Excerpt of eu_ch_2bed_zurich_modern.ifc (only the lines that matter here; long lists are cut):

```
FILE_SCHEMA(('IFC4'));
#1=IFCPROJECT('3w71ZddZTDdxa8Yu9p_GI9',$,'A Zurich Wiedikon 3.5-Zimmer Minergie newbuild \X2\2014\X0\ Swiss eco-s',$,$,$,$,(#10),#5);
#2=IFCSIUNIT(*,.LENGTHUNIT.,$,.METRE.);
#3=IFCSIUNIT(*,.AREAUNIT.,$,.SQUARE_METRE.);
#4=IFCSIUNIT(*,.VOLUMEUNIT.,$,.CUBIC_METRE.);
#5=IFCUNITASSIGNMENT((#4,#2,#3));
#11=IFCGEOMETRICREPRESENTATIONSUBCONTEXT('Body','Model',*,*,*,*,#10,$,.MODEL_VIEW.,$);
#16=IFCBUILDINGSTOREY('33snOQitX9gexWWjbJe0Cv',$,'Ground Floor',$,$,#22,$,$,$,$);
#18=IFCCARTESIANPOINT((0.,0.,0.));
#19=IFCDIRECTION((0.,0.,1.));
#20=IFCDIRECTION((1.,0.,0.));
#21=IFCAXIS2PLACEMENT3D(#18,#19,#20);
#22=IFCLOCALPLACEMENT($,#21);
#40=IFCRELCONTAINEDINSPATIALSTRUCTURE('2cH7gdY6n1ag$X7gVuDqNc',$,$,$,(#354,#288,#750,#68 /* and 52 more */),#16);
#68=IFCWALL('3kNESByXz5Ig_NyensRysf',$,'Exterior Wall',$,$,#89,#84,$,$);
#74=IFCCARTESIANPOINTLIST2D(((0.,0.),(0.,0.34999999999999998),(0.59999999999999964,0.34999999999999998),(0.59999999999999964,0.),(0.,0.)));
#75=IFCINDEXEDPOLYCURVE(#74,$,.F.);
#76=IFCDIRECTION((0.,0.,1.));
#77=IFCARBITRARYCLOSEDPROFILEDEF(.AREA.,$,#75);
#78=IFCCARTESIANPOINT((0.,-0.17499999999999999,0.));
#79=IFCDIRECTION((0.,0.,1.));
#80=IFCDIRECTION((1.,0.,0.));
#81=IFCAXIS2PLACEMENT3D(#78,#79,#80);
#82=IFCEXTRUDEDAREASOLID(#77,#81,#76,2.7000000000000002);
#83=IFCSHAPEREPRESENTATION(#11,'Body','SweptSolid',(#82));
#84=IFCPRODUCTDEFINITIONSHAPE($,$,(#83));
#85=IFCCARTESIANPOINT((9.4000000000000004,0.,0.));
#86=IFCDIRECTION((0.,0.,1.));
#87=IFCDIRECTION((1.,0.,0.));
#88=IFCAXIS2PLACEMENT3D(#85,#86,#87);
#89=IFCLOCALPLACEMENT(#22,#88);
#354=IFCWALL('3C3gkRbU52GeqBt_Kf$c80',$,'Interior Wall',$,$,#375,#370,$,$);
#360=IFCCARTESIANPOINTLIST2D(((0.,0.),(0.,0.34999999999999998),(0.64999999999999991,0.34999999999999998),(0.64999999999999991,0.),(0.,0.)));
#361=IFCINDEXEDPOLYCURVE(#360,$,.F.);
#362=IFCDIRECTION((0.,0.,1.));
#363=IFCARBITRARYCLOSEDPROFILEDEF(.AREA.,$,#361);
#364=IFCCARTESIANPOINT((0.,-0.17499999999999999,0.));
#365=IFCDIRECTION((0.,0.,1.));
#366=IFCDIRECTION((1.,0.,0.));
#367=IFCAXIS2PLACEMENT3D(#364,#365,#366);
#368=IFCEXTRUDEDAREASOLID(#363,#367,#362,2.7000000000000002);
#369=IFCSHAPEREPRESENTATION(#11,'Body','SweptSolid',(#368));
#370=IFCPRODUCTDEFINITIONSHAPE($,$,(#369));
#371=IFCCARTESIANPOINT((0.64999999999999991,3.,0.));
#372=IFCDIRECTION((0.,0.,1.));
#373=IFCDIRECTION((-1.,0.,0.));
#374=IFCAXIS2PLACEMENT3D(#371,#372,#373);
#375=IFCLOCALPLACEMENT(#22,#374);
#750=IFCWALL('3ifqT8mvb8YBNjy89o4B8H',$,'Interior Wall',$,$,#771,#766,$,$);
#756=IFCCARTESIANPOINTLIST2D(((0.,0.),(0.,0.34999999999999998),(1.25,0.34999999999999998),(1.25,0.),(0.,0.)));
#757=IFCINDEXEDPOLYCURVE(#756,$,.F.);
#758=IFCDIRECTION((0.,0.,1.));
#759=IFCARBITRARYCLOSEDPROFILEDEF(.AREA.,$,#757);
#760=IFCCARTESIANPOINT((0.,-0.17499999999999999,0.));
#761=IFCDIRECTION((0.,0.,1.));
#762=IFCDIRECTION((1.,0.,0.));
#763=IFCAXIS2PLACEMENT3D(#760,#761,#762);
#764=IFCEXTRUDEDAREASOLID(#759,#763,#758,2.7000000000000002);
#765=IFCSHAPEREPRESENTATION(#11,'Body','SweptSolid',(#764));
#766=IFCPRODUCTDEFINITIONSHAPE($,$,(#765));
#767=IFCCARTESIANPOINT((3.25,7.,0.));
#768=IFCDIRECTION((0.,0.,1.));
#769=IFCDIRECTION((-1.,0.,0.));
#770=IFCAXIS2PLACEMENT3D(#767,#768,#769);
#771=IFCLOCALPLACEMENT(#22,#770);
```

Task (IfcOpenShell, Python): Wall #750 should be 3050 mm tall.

```python
import ifcopenshell
import ifcopenshell.geom
import ifcopenshell.util.representation
import ifcopenshell.util.shape
import ifcopenshell.util.unit

model = ifcopenshell.open("eu_ch_2bed_zurich_modern.ifc")
unit_scale = ifcopenshell.util.unit.calculate_unit_scale(model)
settings = ifcopenshell.geom.settings()


def volume(element):
    """Net volume in cubic metres, openings subtracted."""
    shape = ifcopenshell.geom.create_shape(settings, element)
    return ifcopenshell.util.shape.get_volume(shape.geometry)


wall = model.by_guid("3ifqT8mvb8YBNjy89o4B8H")
before = volume(wall)

body = ifcopenshell.util.representation.get_representation(wall, "Model", "Body")
solid = body.Items[0]
old_height = solid.Depth
solid.Depth = 3.05 / unit_scale
after = volume(wall)

print(f"height {old_height:g} -> {solid.Depth:g}, volume {before:.3f} -> {after:.3f} m3")

model.write("eu_ch_2bed_zurich_modern_updated.ifc")
```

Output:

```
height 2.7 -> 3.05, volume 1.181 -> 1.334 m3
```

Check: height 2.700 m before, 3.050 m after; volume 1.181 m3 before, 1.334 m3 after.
